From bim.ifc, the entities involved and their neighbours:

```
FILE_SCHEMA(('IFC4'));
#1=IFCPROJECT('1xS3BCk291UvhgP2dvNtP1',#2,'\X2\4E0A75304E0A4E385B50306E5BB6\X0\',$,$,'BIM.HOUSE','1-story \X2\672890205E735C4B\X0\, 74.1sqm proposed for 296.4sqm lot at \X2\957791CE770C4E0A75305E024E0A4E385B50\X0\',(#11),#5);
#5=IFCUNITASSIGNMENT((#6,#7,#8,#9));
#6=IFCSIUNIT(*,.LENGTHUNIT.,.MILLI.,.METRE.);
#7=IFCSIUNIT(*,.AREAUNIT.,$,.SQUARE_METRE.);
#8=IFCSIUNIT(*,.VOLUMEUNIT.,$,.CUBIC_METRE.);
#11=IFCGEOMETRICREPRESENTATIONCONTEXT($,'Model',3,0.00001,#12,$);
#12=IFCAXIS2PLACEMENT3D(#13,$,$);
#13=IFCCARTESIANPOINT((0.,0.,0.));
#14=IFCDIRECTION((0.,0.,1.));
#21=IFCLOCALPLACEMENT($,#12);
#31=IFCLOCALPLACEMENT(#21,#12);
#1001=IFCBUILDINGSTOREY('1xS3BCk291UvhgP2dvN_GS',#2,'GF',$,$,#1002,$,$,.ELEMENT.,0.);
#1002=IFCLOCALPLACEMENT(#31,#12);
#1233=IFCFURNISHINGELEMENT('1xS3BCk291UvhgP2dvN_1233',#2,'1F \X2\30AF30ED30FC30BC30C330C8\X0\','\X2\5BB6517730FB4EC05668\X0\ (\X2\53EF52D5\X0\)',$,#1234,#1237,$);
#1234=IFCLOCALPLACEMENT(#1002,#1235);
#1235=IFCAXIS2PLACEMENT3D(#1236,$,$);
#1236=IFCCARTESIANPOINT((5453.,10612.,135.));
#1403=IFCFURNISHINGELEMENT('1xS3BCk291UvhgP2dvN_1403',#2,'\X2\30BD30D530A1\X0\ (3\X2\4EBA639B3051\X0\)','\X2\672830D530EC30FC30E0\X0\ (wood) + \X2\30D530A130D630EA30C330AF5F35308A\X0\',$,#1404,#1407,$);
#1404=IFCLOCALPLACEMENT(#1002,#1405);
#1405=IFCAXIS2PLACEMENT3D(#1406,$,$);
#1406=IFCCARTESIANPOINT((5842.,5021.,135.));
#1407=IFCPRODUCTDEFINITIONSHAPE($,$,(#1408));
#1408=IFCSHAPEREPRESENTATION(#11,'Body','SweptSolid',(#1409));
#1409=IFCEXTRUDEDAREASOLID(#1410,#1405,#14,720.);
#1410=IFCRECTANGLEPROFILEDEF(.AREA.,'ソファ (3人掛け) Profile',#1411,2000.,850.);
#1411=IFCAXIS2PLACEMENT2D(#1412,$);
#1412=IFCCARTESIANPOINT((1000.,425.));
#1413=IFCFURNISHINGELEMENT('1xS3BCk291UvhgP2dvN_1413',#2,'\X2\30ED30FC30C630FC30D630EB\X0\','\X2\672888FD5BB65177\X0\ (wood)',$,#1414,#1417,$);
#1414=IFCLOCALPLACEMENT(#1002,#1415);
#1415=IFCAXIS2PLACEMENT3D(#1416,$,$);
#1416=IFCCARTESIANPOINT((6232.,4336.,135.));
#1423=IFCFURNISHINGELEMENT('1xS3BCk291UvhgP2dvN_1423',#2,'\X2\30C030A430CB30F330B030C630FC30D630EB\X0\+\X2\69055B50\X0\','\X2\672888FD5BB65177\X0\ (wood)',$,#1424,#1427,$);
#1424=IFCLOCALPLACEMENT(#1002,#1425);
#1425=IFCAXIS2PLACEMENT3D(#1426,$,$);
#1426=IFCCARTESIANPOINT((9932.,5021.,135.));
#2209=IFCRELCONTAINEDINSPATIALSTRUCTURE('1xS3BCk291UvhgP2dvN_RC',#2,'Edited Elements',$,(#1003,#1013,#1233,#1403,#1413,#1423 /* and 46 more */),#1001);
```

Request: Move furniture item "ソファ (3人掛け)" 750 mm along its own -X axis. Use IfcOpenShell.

```python
import ifcopenshell
import ifcopenshell.api.geometry
import ifcopenshell.util.placement
import ifcopenshell.util.unit

model = ifcopenshell.open("bim.ifc")
unit_scale = ifcopenshell.util.unit.calculate_unit_scale(model)

item = model.by_guid("1xS3BCk291UvhgP2dvN_1403")
matrix = ifcopenshell.util.placement.get_local_placement(item.ObjectPlacement)
matrix[:3, 3] -= matrix[:3, 0] * 0.75 / unit_scale
ifcopenshell.api.geometry.edit_object_placement(model, product=item, matrix=matrix, is_si=False)

print(ifcopenshell.util.placement.get_local_placement(item.ObjectPlacement).round(3) + 0.0)

model.write("bim_edited.ifc")
```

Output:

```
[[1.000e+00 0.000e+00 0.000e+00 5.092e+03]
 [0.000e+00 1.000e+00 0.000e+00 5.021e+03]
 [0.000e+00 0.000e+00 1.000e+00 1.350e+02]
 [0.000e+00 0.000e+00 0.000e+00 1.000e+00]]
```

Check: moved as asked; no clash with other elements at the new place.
